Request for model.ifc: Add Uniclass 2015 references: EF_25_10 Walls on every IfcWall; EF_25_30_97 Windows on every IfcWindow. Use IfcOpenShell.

First a look at what the model holds.

```python
import ifcopenshell

model = ifcopenshell.open("model.ifc")
print(model.schema)
print("classifications:", [c.Name for c in model.by_type("IfcClassification")])
for ifc_class in ("IfcDoor", "IfcRoof", "IfcStair", "IfcWall", "IfcWindow"):
    print(ifc_class, len(model.by_type(ifc_class)))
```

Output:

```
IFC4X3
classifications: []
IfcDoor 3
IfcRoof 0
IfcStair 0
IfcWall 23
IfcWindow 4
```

```python
import ifcopenshell
import ifcopenshell.api.classification

model = ifcopenshell.open("model.ifc")

system = ifcopenshell.api.classification.add_classification(model, classification="Uniclass 2015")

codes = {
    "IfcWall": ("EF_25_10", "Walls"),
    "IfcWindow": ("EF_25_30_97", "Windows"),
}
for ifc_class, (code, name) in codes.items():
    products = model.by_type(ifc_class)
    ifcopenshell.api.classification.add_reference(
        model, products=products, classification=system, identification=code, name=name
    )
    print(code, len(products))

model.write("model_v2.ifc")
```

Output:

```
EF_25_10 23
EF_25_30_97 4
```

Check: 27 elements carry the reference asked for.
